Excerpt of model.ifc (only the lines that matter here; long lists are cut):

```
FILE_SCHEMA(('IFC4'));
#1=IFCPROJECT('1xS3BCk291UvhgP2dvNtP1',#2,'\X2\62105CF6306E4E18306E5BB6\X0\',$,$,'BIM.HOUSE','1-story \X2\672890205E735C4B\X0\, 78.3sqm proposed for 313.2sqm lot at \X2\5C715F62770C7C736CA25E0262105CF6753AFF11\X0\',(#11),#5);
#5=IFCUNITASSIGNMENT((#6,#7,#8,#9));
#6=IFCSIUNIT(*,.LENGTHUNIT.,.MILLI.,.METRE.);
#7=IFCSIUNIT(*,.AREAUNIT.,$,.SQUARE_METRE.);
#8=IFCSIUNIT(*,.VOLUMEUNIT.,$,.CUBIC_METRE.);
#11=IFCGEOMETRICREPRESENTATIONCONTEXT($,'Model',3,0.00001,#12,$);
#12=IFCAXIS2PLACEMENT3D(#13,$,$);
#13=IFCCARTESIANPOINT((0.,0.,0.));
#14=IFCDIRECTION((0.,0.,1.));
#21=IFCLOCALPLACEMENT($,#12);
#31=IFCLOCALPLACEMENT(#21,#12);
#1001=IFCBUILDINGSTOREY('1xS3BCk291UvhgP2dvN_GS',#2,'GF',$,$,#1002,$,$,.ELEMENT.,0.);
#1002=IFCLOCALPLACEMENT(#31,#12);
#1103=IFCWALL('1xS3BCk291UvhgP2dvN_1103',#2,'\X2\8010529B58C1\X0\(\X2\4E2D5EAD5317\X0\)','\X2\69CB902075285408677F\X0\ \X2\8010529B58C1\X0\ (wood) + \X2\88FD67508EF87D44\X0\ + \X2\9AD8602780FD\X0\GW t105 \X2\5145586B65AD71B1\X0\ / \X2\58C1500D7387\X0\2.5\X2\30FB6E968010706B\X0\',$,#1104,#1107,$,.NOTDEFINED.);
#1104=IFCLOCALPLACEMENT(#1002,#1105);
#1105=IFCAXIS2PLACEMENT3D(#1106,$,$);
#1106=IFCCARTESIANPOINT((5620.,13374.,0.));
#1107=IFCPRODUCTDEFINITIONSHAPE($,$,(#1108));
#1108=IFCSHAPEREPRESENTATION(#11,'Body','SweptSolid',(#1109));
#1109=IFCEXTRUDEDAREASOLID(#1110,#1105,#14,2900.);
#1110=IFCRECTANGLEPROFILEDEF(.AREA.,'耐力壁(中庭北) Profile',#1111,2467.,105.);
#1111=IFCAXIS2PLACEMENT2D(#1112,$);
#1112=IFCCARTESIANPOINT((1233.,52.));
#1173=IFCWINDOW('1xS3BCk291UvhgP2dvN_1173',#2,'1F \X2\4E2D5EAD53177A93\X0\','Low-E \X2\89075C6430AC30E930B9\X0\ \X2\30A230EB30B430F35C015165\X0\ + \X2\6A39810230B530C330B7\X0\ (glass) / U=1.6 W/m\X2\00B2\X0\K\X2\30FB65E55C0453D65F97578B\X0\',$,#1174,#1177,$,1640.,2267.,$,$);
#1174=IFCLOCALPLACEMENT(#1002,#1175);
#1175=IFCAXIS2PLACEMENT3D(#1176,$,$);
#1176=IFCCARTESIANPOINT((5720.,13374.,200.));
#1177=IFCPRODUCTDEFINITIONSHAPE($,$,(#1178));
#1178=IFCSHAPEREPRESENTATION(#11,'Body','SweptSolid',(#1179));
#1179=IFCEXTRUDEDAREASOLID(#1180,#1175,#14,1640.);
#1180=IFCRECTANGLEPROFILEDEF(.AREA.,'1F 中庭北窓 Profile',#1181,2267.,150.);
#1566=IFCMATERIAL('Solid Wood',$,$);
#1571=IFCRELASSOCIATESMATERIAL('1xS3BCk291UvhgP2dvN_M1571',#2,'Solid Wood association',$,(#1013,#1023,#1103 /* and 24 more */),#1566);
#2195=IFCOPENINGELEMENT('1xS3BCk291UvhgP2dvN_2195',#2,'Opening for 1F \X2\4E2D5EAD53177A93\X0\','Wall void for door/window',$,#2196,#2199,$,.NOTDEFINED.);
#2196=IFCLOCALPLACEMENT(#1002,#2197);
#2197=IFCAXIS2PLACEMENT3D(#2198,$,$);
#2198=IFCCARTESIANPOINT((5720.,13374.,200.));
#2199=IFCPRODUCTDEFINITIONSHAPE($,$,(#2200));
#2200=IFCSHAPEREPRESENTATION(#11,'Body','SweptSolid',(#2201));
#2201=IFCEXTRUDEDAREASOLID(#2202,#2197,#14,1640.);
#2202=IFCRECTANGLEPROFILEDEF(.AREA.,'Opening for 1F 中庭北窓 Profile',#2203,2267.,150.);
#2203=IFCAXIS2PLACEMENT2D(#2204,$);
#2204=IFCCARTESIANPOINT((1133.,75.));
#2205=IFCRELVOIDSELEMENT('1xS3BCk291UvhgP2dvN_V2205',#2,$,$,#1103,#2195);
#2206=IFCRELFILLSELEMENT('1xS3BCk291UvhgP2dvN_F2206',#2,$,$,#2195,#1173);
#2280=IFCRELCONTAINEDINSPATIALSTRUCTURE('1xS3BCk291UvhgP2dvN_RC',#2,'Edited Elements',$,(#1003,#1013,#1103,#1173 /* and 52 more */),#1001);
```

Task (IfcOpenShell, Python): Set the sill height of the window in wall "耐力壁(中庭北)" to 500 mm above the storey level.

```python
import numpy as np
import ifcopenshell
import ifcopenshell.api.geometry
import ifcopenshell.geom
import ifcopenshell.util.element
import ifcopenshell.util.placement
import ifcopenshell.util.shape
import ifcopenshell.util.unit

model = ifcopenshell.open("model.ifc")
unit_scale = ifcopenshell.util.unit.calculate_unit_scale(model)

window = model.by_guid("1xS3BCk291UvhgP2dvN_1173")
opening = window.FillsVoids[0].RelatingOpeningElement
storey = ifcopenshell.util.element.get_container(window, ifc_class="IfcBuildingStorey")
level = ifcopenshell.util.placement.get_local_placement(storey.ObjectPlacement)[2, 3]

# The opening's origin need not be at the sill, so measure its lowest point.
shape = ifcopenshell.geom.create_shape(ifcopenshell.geom.settings(), opening)
bottom = ifcopenshell.util.shape.get_shape_bottom_elevation(shape, shape.geometry) / unit_scale
dz = level + 0.5 / unit_scale - bottom

shift = np.array([0.0, 0.0, dz])
# The window is not placed relative to its opening, so move both.
for product in (opening, window):
    matrix = ifcopenshell.util.placement.get_local_placement(product.ObjectPlacement)
    matrix[:3, 3] += shift
    ifcopenshell.api.geometry.edit_object_placement(model, product=product, matrix=matrix, is_si=False)

print(f"moved by {dz * unit_scale:+.3f} m")

model.write("model_rev.ifc")
```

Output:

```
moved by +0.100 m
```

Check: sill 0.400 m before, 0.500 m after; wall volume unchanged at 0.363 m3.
